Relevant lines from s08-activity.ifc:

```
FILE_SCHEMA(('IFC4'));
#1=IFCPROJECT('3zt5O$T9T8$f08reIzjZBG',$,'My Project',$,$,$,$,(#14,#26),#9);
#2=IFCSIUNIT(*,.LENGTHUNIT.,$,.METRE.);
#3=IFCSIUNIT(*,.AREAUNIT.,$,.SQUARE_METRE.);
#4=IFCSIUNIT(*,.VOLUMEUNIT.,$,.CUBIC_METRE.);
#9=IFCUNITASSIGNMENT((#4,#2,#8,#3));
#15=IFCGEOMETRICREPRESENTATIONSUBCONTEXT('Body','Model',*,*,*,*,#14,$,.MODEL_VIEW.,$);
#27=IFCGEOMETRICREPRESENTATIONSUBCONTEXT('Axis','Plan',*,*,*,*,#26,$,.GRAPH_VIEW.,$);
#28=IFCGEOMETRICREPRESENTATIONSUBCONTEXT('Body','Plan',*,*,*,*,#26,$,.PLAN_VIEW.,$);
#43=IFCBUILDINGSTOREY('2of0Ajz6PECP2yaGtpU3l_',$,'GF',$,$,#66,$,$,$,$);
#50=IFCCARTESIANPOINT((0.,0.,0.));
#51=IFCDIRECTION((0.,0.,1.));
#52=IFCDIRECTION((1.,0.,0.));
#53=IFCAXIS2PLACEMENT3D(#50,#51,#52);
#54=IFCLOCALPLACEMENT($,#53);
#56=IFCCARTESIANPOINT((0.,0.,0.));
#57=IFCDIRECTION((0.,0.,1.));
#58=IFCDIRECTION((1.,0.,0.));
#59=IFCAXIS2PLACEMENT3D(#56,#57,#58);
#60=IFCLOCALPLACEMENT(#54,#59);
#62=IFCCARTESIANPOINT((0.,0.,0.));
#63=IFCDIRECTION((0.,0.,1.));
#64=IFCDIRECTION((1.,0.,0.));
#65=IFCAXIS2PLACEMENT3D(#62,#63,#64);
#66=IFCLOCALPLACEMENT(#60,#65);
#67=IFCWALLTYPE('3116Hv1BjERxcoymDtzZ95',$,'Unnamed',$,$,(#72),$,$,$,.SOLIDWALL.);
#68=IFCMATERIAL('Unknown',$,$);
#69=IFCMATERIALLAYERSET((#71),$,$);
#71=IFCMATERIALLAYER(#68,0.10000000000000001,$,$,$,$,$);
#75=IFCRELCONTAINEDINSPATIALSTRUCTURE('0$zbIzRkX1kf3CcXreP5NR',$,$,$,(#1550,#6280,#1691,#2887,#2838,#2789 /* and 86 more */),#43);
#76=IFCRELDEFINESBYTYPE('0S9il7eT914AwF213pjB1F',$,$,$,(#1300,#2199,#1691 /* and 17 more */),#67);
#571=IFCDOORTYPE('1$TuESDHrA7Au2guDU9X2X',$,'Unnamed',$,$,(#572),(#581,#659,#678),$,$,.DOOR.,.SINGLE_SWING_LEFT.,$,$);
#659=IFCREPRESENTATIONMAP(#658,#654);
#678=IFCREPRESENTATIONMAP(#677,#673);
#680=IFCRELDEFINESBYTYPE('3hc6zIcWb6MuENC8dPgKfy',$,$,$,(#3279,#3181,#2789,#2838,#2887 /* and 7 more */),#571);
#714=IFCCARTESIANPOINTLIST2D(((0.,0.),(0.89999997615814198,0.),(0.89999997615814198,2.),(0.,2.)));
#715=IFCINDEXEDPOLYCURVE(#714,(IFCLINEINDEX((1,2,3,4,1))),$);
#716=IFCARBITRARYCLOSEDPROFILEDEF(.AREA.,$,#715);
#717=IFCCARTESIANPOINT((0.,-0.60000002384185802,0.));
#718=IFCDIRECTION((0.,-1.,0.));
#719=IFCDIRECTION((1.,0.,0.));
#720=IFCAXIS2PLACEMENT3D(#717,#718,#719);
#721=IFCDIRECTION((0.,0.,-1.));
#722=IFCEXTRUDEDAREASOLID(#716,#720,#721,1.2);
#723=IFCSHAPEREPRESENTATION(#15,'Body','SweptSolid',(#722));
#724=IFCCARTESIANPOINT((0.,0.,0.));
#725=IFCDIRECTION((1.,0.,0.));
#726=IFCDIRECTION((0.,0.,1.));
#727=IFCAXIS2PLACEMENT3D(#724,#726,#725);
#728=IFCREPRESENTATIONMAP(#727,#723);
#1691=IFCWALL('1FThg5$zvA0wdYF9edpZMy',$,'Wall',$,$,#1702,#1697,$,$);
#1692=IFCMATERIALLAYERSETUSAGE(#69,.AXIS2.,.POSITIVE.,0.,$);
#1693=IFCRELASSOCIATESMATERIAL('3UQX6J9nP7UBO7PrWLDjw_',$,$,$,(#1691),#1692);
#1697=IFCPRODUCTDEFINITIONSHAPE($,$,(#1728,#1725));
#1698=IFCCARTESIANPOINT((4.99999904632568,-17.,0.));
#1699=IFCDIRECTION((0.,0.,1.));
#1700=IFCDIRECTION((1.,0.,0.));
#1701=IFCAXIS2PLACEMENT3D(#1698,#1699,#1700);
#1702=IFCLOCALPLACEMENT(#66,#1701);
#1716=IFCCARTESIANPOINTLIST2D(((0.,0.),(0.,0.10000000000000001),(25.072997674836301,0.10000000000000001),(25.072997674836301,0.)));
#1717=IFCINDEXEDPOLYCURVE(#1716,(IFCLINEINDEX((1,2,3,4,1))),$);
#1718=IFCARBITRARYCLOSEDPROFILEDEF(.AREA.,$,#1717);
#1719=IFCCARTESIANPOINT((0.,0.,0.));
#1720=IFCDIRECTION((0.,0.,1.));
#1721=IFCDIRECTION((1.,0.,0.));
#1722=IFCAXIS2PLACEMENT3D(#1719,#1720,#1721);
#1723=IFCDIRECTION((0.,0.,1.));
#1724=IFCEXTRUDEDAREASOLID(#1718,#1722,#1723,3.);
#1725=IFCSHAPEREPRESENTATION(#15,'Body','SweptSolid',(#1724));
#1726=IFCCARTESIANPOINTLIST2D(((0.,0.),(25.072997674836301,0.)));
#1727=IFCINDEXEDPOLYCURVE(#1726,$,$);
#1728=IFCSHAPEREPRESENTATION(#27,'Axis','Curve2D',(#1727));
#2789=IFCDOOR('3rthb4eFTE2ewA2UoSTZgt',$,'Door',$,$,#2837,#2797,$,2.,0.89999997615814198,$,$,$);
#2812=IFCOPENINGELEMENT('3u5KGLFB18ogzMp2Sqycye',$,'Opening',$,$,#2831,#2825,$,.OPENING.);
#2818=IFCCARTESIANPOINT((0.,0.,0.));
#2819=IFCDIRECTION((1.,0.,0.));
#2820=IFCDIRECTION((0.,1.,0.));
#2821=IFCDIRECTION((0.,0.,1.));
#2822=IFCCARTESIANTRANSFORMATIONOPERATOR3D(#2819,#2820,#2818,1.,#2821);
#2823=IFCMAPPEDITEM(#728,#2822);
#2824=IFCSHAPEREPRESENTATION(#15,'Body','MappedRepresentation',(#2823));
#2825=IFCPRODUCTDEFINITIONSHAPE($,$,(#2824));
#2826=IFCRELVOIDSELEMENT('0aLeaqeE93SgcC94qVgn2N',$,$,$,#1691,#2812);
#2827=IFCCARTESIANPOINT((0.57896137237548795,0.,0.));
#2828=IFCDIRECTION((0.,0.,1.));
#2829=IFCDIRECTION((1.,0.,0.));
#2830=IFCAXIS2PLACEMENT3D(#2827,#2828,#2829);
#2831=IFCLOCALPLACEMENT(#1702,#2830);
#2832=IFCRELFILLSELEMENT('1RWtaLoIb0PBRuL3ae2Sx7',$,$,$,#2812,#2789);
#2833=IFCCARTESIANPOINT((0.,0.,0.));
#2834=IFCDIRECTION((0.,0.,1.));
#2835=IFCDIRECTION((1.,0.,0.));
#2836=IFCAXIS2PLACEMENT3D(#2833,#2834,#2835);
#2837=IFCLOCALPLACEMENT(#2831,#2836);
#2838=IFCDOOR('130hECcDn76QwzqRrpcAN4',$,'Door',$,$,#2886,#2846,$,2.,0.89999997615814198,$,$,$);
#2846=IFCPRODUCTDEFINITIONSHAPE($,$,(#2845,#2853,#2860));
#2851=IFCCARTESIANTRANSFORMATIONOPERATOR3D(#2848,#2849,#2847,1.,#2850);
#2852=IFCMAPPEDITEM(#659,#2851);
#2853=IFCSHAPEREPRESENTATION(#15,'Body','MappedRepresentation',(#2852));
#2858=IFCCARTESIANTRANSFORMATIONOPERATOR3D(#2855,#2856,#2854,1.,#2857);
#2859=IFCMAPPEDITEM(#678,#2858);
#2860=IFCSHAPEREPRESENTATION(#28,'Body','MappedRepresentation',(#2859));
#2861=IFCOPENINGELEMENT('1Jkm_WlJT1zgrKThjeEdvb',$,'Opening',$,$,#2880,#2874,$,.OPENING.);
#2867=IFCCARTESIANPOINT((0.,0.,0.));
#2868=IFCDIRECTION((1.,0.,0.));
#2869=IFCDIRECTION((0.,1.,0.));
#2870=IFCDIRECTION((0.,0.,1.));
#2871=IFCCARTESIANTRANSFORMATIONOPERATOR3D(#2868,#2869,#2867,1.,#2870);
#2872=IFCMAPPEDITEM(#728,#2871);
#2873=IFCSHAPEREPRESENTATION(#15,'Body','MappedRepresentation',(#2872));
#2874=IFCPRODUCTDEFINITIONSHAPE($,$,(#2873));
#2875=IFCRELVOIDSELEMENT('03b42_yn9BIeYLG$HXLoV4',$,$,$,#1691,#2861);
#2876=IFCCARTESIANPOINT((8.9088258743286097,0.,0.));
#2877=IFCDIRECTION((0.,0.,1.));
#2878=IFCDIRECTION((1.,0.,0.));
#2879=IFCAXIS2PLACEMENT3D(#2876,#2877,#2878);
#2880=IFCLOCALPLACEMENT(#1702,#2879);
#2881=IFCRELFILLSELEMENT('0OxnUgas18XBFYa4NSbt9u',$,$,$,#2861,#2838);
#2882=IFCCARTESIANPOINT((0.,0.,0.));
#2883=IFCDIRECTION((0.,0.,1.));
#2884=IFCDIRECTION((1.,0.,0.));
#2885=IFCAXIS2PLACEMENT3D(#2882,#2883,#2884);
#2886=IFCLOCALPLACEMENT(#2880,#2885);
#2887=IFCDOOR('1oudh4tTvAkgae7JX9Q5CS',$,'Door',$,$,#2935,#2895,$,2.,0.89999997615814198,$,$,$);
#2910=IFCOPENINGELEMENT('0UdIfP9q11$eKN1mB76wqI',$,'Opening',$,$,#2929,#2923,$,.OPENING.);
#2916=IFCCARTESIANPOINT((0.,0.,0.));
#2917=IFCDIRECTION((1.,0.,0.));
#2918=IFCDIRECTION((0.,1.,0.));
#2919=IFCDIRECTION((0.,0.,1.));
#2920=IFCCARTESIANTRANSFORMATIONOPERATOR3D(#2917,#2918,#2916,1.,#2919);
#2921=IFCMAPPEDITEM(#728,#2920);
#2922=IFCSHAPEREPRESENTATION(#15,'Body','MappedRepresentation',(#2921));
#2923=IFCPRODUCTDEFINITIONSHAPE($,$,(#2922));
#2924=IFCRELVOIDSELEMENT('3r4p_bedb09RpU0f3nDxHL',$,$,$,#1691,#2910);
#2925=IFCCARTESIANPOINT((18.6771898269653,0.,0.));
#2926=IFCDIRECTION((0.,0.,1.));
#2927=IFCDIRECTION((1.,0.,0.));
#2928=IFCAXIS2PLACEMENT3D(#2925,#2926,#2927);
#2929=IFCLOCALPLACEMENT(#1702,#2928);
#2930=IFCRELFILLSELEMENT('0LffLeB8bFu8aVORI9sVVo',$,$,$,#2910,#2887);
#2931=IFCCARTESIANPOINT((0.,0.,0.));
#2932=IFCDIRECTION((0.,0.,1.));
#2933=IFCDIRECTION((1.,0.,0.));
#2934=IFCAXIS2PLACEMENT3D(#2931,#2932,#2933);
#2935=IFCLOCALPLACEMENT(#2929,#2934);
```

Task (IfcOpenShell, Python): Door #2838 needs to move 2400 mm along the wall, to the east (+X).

```python
import ifcopenshell
import ifcopenshell.api.geometry
import ifcopenshell.util.placement

model = ifcopenshell.open("s08-activity.ifc")

door = model.by_id(2838)
opening = door.FillsVoids[0].RelatingOpeningElement
wall = opening.VoidsElements[0].RelatingBuildingElement

wall_matrix = ifcopenshell.util.placement.get_local_placement(wall.ObjectPlacement)
shift = wall_matrix[:3, 0] * 2.4
before = ifcopenshell.util.placement.get_local_placement(door.ObjectPlacement)[:3, 3].copy()

# The door is placed relative to its opening, so it follows when the opening moves.
matrix = ifcopenshell.util.placement.get_local_placement(opening.ObjectPlacement)
matrix[:3, 3] += shift
ifcopenshell.api.geometry.edit_object_placement(
    model, product=opening, matrix=matrix, is_si=False, should_transform_children=True
)

after = ifcopenshell.util.placement.get_local_placement(door.ObjectPlacement)[:3, 3]
print("door moved by", (after - before).round(3) + 0.0)

model.write("s08-activity_rev.ifc")
```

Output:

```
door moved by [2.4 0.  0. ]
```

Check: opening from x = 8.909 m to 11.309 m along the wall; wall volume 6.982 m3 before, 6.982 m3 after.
